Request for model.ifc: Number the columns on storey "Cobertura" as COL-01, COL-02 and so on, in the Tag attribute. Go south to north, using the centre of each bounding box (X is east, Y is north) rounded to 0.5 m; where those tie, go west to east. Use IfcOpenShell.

First a look at what the model holds.

```python
import ifcopenshell
import ifcopenshell.util.element
import ifcopenshell.util.placement

model = ifcopenshell.open("model.ifc")
print(model.schema)
storey = next(s for s in model.by_type("IfcBuildingStorey") if s.Name == "Cobertura")
columns = [e for e in ifcopenshell.util.element.get_decomposition(storey) if e.is_a("IfcColumn")]
for e in sorted(columns, key=lambda e: e.id()):
    origin = ifcopenshell.util.placement.get_local_placement(e.ObjectPlacement)[:3, 3]
    print(e.id(), e.Tag, e.Name, origin.round(2) + 0.0, sep=" | ")
```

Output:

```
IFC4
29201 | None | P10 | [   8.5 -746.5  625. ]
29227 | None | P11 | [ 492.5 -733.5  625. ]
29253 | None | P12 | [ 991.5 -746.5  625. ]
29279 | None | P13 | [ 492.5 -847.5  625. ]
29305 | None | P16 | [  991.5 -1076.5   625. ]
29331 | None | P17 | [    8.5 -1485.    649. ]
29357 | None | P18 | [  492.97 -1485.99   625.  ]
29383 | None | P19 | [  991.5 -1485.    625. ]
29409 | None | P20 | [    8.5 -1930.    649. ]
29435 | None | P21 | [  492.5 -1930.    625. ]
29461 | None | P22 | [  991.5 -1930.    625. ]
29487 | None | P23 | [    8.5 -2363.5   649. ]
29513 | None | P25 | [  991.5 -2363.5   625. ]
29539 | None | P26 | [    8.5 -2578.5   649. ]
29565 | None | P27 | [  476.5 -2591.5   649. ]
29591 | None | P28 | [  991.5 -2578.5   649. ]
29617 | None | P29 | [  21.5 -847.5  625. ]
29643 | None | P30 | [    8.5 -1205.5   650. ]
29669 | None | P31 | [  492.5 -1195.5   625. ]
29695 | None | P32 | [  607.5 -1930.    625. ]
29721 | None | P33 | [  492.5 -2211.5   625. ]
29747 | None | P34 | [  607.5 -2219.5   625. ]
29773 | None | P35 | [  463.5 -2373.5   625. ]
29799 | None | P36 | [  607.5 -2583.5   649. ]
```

```python
import ifcopenshell
import ifcopenshell.geom
import ifcopenshell.util.element
import ifcopenshell.util.shape

model = ifcopenshell.open("model.ifc")
settings = ifcopenshell.geom.settings()
settings.set("use-world-coords", True)


def centre(element):
    shape = ifcopenshell.geom.create_shape(settings, element)
    return ifcopenshell.util.shape.get_bbox_centroid(shape.geometry)


storey = next(s for s in model.by_type("IfcBuildingStorey") if s.Name == "Cobertura")
columns = [e for e in ifcopenshell.util.element.get_decomposition(storey) if e.is_a("IfcColumn")]

# Insertion points can sit at a corner or the storey origin, so sort by the geometry (in metres).
centres = {e: centre(e) for e in columns}
columns.sort(key=lambda e: (round(centres[e][1] / 0.5), centres[e][0]))

for i, e in enumerate(columns, start=1):
    number = f"COL-{i:02d}"
    e.Tag = number
    print(e.id(), number)

model.write("model_v2.ifc")
```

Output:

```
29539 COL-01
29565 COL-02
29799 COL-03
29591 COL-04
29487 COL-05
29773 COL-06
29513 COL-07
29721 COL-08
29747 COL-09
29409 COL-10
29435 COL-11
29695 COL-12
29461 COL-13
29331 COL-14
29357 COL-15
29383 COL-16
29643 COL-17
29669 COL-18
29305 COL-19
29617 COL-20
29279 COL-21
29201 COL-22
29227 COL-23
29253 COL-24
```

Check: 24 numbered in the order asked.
